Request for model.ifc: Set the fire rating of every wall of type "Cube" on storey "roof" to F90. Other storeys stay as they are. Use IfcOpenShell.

First a look at what the model holds.

```python
import ifcopenshell
import ifcopenshell.util.element

model = ifcopenshell.open("model.ifc")
print(model.schema)
storey = next(s for s in model.by_type("IfcBuildingStorey") if s.Name == "roof")
walls = [e for e in ifcopenshell.util.element.get_decomposition(storey) if e.is_a("IfcWall")]
seen = {}
for e in walls:
    element_type = ifcopenshell.util.element.get_type(e)
    key = (element_type.Name if element_type != e and element_type else None, ifcopenshell.util.element.get_pset(e, "Pset_WallCommon", "FireRating"))
    seen[key] = seen.get(key, 0) + 1
for (name, value), count in sorted(seen.items(), key=str):
    print(count, "x", name, "|", value)
```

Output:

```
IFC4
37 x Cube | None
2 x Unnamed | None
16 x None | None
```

```python
import ifcopenshell
import ifcopenshell.api.pset
import ifcopenshell.util.element

model = ifcopenshell.open("model.ifc")

storey = next(s for s in model.by_type("IfcBuildingStorey") if s.Name == "roof")
walls = [e for e in ifcopenshell.util.element.get_decomposition(storey) if e.is_a("IfcWall")]

count = 0
for e in walls:
    element_type = ifcopenshell.util.element.get_type(e)
    if element_type in (None, e) or element_type.Name != "Cube":
        continue
    # add_pset returns the element's existing set when there is one.
    pset = ifcopenshell.api.pset.add_pset(model, product=e, name="Pset_WallCommon")
    ifcopenshell.api.pset.edit_pset(model, pset=pset, properties={"FireRating": "F90"})
    count += 1

print(count, "walls updated")

model.write("model_rev.ifc")
```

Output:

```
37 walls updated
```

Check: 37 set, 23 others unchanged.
